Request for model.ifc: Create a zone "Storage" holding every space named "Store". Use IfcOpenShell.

First a look at what the model holds.

```python
import ifcopenshell

model = ifcopenshell.open("model.ifc")
print(model.schema)
seen = {}
for space in model.by_type("IfcSpace"):
    seen[space.LongName] = seen.get(space.LongName, 0) + 1
for name, count in sorted(seen.items(), key=str):
    print(count, "x", name)
print("zones:", [z.Name for z in model.by_type("IfcZone")][:20])
```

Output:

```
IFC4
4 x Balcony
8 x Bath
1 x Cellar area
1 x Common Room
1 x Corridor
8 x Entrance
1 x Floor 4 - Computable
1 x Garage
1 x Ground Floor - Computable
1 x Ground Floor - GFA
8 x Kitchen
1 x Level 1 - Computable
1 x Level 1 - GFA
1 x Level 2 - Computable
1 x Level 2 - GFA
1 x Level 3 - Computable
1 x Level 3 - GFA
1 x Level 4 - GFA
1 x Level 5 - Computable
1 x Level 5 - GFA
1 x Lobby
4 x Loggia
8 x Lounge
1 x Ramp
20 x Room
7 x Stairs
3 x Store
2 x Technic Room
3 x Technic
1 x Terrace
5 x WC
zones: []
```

```python
import ifcopenshell
import ifcopenshell.api.group
import ifcopenshell.api.root

model = ifcopenshell.open("model.ifc")

names = {"Store"}
spaces = [s for s in model.by_type("IfcSpace") if s.LongName in names]

zone = ifcopenshell.api.root.create_entity(model, ifc_class="IfcZone", name="Storage")
ifcopenshell.api.group.assign_group(model, products=spaces, group=zone)
print(len(spaces), "spaces in", zone.Name)

model.write("model_rev.ifc")
```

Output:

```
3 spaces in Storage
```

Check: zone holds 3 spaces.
